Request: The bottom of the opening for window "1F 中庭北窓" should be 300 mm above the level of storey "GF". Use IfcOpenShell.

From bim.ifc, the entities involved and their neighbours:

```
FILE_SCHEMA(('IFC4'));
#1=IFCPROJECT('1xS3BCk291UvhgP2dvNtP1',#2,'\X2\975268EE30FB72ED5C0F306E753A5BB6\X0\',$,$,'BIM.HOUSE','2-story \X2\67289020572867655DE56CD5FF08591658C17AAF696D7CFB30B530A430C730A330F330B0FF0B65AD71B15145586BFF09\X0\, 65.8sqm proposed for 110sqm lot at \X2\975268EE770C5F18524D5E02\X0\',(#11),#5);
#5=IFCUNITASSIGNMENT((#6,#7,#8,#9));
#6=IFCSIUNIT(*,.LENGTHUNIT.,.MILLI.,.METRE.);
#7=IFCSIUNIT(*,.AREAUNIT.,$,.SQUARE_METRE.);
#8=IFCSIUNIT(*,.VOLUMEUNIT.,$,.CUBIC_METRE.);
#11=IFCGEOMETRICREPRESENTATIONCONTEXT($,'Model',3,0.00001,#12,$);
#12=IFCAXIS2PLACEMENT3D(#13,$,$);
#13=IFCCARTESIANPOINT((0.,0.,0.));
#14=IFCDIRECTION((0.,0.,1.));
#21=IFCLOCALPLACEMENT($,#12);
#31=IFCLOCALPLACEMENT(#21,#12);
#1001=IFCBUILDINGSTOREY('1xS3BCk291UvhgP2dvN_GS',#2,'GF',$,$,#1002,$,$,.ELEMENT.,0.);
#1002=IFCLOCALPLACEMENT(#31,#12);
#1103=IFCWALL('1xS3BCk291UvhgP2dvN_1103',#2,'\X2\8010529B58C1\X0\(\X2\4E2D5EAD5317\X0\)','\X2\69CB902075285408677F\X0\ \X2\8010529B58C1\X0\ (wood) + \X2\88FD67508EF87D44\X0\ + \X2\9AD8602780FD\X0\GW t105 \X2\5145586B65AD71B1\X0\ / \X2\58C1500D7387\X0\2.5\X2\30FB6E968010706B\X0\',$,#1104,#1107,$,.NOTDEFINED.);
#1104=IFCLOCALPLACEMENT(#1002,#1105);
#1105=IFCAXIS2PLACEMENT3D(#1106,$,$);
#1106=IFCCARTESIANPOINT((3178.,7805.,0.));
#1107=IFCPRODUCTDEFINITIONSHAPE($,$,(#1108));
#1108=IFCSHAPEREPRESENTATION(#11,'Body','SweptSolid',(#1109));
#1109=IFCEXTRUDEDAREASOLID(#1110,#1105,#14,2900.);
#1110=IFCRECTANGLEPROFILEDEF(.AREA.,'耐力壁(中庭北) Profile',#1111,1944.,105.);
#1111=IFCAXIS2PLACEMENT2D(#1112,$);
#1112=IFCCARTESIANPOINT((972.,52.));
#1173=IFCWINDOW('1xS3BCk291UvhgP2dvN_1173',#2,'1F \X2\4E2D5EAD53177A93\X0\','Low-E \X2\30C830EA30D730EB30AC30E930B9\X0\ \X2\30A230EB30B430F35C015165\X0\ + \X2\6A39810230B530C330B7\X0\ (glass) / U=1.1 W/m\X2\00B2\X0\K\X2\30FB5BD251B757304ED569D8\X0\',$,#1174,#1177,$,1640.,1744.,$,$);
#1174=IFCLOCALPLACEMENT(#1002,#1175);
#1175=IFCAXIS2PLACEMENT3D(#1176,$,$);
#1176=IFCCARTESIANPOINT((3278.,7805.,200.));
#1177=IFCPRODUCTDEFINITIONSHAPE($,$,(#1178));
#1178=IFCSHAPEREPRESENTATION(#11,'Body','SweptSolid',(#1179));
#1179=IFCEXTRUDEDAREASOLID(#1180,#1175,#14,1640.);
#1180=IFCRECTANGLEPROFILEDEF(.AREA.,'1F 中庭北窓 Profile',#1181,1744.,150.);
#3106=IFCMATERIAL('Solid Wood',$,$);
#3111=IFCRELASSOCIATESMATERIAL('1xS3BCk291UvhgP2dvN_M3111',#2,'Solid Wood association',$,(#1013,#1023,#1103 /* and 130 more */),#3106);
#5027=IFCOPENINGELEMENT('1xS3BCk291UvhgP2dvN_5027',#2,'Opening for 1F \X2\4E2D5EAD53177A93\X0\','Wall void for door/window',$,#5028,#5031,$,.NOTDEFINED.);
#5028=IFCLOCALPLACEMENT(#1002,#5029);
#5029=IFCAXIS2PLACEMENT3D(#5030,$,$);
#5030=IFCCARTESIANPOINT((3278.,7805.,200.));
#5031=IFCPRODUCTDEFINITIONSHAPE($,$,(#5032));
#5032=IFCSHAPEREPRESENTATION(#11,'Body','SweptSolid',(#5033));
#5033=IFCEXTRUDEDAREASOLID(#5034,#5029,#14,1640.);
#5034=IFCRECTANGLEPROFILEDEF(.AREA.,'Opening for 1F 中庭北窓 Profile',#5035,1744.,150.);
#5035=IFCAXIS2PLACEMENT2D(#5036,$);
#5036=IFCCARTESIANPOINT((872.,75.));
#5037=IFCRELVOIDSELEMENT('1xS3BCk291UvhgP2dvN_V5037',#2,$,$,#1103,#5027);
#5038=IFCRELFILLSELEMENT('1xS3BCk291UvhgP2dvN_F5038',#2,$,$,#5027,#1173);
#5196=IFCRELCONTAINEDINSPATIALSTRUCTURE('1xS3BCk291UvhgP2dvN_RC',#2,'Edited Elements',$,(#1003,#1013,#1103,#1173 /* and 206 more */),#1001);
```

```python
import numpy as np
import ifcopenshell
import ifcopenshell.api.geometry
import ifcopenshell.geom
import ifcopenshell.util.element
import ifcopenshell.util.placement
import ifcopenshell.util.shape
import ifcopenshell.util.unit

model = ifcopenshell.open("bim.ifc")
unit_scale = ifcopenshell.util.unit.calculate_unit_scale(model)

window = model.by_id(1173)
opening = window.FillsVoids[0].RelatingOpeningElement
storey = ifcopenshell.util.element.get_container(window, ifc_class="IfcBuildingStorey")
level = ifcopenshell.util.placement.get_local_placement(storey.ObjectPlacement)[2, 3]

# The opening's origin need not be at the sill, so measure its lowest point.
shape = ifcopenshell.geom.create_shape(ifcopenshell.geom.settings(), opening)
bottom = ifcopenshell.util.shape.get_shape_bottom_elevation(shape, shape.geometry) / unit_scale
dz = level + 0.3 / unit_scale - bottom

shift = np.array([0.0, 0.0, dz])
# The window is not placed relative to its opening, so move both.
for product in (opening, window):
    matrix = ifcopenshell.util.placement.get_local_placement(product.ObjectPlacement)
    matrix[:3, 3] += shift
    ifcopenshell.api.geometry.edit_object_placement(model, product=product, matrix=matrix, is_si=False)

print(f"moved by {dz * unit_scale:+.3f} m")

model.write("bim-out.ifc")
```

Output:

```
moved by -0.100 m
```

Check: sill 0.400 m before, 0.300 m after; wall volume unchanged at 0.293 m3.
